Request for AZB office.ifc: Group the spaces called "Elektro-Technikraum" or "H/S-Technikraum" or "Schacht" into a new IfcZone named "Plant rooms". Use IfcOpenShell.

First a look at what the model holds.

```python
import ifcopenshell

model = ifcopenshell.open("AZB office.ifc")
print(model.schema)
seen = {}
for space in model.by_type("IfcSpace"):
    seen[space.LongName] = seen.get(space.LongName, 0) + 1
for name, count in sorted(seen.items(), key=str):
    print(count, "x", name)
print("zones:", [z.Name for z in model.by_type("IfcZone")][:20])
```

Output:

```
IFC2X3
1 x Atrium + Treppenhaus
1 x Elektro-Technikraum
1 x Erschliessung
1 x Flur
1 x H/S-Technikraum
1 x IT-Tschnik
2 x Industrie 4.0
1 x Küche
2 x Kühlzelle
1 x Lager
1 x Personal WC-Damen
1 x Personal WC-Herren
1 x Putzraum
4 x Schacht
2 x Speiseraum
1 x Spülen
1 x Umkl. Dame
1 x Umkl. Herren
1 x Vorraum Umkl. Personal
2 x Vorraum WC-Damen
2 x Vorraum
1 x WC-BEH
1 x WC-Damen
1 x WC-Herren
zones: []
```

```python
import ifcopenshell
import ifcopenshell.api.group
import ifcopenshell.api.root

model = ifcopenshell.open("AZB office.ifc")

names = {"Elektro-Technikraum", "H/S-Technikraum", "Schacht"}
spaces = [s for s in model.by_type("IfcSpace") if s.LongName in names]

zone = ifcopenshell.api.root.create_entity(model, ifc_class="IfcZone", name="Plant rooms")
ifcopenshell.api.group.assign_group(model, products=spaces, group=zone)
print(len(spaces), "spaces in", zone.Name)

model.write("AZB office_rev.ifc")
```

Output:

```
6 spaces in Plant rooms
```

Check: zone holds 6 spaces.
